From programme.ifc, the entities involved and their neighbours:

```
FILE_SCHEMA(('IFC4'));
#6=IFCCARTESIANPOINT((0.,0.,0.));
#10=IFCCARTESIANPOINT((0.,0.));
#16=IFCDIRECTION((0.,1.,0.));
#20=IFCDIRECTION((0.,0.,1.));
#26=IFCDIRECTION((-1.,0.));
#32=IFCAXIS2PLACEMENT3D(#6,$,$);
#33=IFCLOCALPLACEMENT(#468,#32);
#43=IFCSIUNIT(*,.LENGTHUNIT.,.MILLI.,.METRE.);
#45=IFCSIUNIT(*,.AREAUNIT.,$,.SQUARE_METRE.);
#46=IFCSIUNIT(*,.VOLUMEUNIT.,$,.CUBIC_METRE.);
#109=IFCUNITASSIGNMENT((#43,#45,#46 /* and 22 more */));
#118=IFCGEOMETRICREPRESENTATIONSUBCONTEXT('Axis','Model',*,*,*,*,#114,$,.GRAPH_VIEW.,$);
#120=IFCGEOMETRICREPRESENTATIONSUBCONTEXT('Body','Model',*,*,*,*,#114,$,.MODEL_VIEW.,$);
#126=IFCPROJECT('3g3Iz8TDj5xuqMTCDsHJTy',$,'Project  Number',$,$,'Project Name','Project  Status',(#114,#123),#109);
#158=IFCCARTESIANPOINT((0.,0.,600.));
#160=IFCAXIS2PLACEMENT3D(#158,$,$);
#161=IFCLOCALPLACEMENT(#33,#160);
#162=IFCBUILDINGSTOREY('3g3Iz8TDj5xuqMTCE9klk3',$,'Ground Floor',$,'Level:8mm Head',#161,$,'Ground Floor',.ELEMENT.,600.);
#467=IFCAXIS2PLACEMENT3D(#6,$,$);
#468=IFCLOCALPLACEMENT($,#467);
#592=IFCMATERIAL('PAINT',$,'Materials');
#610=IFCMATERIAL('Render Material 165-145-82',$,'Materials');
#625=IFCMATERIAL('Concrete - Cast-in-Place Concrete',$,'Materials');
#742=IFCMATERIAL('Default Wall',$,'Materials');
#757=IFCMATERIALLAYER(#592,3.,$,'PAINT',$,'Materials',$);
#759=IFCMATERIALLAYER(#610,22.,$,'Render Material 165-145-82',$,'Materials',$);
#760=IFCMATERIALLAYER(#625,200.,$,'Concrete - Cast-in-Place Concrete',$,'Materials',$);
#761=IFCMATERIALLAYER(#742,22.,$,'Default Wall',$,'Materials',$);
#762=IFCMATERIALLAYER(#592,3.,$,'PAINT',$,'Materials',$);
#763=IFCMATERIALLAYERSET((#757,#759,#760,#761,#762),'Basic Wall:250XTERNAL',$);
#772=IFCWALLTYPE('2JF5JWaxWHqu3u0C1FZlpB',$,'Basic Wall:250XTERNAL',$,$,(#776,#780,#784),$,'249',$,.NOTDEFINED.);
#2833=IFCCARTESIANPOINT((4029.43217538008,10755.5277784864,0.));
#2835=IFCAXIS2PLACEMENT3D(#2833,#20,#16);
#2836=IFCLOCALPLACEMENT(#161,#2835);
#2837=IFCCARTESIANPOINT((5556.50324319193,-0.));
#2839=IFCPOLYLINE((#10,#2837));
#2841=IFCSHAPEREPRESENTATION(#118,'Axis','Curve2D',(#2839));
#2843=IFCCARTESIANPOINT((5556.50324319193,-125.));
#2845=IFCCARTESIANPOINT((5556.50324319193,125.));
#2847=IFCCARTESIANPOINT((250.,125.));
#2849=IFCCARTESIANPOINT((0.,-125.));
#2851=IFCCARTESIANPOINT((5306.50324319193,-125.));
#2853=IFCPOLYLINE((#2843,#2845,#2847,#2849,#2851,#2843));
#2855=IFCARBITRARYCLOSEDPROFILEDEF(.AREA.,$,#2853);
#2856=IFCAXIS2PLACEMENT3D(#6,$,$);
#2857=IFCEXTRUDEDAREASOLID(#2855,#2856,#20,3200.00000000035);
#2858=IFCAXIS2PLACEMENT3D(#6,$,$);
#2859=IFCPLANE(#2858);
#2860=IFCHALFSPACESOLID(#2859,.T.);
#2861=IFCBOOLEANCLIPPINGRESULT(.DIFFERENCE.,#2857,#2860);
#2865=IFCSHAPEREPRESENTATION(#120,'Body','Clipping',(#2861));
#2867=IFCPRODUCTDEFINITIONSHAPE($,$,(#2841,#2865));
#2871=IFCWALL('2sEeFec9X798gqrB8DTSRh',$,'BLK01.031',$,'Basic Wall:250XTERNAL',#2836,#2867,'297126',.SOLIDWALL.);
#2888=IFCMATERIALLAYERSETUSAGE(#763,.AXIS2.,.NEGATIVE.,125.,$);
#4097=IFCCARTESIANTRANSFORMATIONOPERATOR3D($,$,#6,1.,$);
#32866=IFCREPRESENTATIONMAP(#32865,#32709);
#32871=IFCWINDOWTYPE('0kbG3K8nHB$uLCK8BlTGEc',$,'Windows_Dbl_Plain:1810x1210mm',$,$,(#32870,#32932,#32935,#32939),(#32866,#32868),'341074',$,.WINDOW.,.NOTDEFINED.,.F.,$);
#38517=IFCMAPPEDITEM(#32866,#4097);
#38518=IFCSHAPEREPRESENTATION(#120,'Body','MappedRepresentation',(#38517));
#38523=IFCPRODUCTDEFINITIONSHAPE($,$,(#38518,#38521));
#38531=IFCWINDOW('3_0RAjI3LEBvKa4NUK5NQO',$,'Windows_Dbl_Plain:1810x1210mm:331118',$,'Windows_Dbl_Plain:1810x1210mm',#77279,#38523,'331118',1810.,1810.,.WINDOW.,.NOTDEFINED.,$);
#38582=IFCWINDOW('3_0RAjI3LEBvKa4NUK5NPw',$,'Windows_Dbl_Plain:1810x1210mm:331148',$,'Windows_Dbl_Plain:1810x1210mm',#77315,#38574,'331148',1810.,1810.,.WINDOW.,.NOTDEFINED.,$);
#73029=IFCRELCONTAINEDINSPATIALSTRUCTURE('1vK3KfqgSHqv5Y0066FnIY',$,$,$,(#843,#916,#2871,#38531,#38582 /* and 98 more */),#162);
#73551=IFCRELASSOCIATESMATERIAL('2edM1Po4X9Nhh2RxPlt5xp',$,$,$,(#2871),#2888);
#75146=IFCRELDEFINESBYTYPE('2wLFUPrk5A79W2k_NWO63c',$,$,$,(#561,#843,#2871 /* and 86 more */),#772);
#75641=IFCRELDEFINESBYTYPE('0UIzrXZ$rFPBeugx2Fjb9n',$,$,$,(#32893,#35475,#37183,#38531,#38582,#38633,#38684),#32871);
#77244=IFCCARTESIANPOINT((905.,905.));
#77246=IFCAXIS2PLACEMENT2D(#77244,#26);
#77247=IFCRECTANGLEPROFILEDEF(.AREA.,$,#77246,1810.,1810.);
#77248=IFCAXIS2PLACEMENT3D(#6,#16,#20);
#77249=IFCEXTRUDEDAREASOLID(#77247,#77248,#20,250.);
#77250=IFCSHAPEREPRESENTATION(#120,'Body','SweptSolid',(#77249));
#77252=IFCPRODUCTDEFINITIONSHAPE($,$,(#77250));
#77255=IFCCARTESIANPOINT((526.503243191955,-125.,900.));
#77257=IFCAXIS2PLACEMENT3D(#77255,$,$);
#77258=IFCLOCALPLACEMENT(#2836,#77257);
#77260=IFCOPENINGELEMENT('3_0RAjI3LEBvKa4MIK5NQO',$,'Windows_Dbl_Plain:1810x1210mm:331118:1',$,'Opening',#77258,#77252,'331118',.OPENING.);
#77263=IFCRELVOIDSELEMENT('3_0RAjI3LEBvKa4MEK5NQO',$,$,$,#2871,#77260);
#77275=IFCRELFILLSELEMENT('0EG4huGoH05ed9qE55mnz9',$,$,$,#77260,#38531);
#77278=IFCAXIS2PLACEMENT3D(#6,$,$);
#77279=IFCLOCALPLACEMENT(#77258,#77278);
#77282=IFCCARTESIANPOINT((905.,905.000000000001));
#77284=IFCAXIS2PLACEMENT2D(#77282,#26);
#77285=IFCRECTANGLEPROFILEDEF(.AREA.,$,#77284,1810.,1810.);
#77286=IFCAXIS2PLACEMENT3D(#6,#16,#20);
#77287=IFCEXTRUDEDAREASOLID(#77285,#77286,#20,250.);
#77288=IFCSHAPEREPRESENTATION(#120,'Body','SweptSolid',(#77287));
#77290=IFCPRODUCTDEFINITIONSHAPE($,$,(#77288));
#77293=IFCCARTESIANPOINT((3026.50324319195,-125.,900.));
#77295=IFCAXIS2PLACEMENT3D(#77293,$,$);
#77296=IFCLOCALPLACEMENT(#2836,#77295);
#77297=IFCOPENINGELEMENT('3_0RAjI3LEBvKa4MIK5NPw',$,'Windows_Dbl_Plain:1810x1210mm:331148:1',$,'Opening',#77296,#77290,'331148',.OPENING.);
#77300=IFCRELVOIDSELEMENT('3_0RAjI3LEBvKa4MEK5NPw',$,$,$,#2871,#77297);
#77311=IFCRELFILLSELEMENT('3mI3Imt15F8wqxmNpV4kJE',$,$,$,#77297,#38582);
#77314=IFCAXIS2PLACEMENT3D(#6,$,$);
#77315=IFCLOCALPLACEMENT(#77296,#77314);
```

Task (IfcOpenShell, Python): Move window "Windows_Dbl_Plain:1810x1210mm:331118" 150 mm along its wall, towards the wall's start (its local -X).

```python
import ifcopenshell
import ifcopenshell.api.geometry
import ifcopenshell.util.placement
import ifcopenshell.util.unit

model = ifcopenshell.open("programme.ifc")
unit_scale = ifcopenshell.util.unit.calculate_unit_scale(model)

window = model.by_guid("3_0RAjI3LEBvKa4NUK5NQO")
opening = window.FillsVoids[0].RelatingOpeningElement
wall = opening.VoidsElements[0].RelatingBuildingElement

wall_matrix = ifcopenshell.util.placement.get_local_placement(wall.ObjectPlacement)
shift = wall_matrix[:3, 0] * -0.15 / unit_scale
before = ifcopenshell.util.placement.get_local_placement(window.ObjectPlacement)[:3, 3].copy()

# The window is placed relative to its opening, so it follows when the opening moves.
matrix = ifcopenshell.util.placement.get_local_placement(opening.ObjectPlacement)
matrix[:3, 3] += shift
ifcopenshell.api.geometry.edit_object_placement(
    model, product=opening, matrix=matrix, is_si=False, should_transform_children=True
)

after = ifcopenshell.util.placement.get_local_placement(window.ObjectPlacement)[:3, 3]
print("window moved by", (after - before).round(3) + 0.0)

model.write("programme_rev.ifc")
```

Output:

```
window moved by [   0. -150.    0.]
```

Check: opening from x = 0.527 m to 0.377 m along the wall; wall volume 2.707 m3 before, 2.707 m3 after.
